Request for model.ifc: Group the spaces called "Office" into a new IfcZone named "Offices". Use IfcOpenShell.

First a look at what the model holds.

```python
import ifcopenshell

model = ifcopenshell.open("model.ifc")
print(model.schema)
seen = {}
for space in model.by_type("IfcSpace"):
    seen[space.LongName] = seen.get(space.LongName, 0) + 1
for name, count in sorted(seen.items(), key=str):
    print(count, "x", name)
print("zones:", [z.Name for z in model.by_type("IfcZone")][:20])
```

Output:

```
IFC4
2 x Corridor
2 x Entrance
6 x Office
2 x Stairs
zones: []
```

```python
import ifcopenshell
import ifcopenshell.api.group
import ifcopenshell.api.root

model = ifcopenshell.open("model.ifc")

names = {"Office"}
spaces = [s for s in model.by_type("IfcSpace") if s.LongName in names]

zone = ifcopenshell.api.root.create_entity(model, ifc_class="IfcZone", name="Offices")
ifcopenshell.api.group.assign_group(model, products=spaces, group=zone)
print(len(spaces), "spaces in", zone.Name)

model.write("model_updated.ifc")
```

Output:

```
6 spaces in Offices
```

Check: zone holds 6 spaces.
